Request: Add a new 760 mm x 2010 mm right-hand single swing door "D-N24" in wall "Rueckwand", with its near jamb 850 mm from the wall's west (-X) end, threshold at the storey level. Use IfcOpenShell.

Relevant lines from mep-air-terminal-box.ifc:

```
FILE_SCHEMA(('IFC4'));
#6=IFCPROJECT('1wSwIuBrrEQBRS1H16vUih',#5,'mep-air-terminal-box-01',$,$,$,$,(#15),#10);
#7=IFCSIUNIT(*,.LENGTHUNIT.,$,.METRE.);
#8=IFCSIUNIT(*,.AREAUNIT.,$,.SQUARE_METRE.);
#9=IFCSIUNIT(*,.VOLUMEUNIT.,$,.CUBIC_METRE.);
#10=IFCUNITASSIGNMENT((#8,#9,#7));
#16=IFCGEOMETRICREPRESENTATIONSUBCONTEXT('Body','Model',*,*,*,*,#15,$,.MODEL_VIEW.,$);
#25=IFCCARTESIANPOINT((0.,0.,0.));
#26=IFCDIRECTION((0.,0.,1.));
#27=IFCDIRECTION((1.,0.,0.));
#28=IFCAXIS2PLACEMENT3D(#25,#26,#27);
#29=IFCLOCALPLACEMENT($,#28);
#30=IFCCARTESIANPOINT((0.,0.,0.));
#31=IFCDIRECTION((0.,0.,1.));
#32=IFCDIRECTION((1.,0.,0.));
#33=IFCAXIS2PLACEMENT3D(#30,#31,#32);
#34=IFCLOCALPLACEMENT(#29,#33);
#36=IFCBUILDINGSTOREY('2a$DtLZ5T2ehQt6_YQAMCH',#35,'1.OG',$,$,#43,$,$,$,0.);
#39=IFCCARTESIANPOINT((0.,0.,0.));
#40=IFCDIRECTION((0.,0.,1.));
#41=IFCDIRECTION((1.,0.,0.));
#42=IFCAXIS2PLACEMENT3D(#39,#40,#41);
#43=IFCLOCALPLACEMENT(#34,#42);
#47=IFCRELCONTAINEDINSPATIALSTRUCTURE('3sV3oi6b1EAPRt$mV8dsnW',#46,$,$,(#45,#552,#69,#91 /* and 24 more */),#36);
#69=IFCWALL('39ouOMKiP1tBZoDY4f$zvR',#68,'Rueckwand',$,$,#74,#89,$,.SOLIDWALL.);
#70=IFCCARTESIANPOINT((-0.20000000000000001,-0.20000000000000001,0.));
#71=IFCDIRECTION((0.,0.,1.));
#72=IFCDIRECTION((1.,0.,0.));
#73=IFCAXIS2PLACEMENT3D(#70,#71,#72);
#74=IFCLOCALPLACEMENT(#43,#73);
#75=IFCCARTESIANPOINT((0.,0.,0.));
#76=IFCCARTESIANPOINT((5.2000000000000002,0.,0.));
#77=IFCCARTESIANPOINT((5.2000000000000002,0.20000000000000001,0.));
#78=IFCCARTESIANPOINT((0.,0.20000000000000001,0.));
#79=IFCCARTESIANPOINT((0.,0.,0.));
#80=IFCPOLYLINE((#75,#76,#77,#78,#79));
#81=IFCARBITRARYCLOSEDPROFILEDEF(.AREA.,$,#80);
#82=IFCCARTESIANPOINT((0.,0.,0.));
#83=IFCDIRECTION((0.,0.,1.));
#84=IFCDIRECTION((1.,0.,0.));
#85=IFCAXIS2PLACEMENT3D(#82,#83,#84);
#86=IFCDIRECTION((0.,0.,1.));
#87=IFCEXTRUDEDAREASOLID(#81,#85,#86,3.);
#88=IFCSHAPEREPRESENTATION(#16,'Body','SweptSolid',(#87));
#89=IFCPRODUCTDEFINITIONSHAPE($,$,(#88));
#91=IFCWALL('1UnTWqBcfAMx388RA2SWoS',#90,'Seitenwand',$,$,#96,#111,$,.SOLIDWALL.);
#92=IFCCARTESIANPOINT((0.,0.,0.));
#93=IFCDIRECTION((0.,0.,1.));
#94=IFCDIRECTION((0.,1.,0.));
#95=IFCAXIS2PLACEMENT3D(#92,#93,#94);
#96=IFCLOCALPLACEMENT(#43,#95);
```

```python
import numpy as np
import ifcopenshell
import ifcopenshell.api.feature
import ifcopenshell.api.geometry
import ifcopenshell.api.root
import ifcopenshell.api.spatial
import ifcopenshell.geom
import ifcopenshell.util.element
import ifcopenshell.util.placement
import ifcopenshell.util.representation
import ifcopenshell.util.shape
import ifcopenshell.util.unit

model = ifcopenshell.open("mep-air-terminal-box.ifc")
unit_scale = ifcopenshell.util.unit.calculate_unit_scale(model)
settings = ifcopenshell.geom.settings()


def volume(element):
    """Net volume in cubic metres, openings subtracted."""
    shape = ifcopenshell.geom.create_shape(settings, element)
    return ifcopenshell.util.shape.get_volume(shape.geometry)


wall = model.by_id(69)
storey = ifcopenshell.util.element.get_container(wall, ifc_class="IfcBuildingStorey")
context = ifcopenshell.util.representation.get_context(model, "Model", "Body", "MODEL_VIEW")
before = volume(wall)

width, height, from_end, sill = 0.76, 2.01, 0.85, 0.0  # metres

# The wall runs along its own X axis, and the end named is its -X end.
wall_shape = ifcopenshell.geom.create_shape(settings, wall)
x, y, z = ifcopenshell.util.shape.get_vertices(wall_shape.geometry).T
start = x.min() + from_end
face, thickness = float(y.min()), float(y.max() - y.min())
wall_matrix = ifcopenshell.util.placement.get_local_placement(wall.ObjectPlacement)
level = ifcopenshell.util.placement.get_local_placement(storey.ObjectPlacement)[2, 3]


def in_wall(x, y):
    """Placement at x, y metres in the wall's axes, at sill height."""
    matrix = wall_matrix.copy()
    matrix[:, 3] = wall_matrix @ np.array([x / unit_scale, y / unit_scale, 0.0, 1.0])
    matrix[2, 3] = level + sill / unit_scale
    return matrix


# Opening: a box that overshoots both wall faces by 50 mm.
opening = ifcopenshell.api.root.create_entity(model, ifc_class="IfcOpeningElement", predefined_type="OPENING")
box = ifcopenshell.api.geometry.add_wall_representation(
    model, context=context, length=width, height=height, thickness=thickness + 0.1
)
ifcopenshell.api.geometry.assign_representation(model, product=opening, representation=box)
ifcopenshell.api.geometry.edit_object_placement(model, product=opening, matrix=in_wall(start, face - 0.05), is_si=False)
ifcopenshell.api.feature.add_feature(model, feature=opening, element=wall)

door = ifcopenshell.api.root.create_entity(model, ifc_class="IfcDoor", name="D-N24", predefined_type="DOOR")
door.OverallWidth, door.OverallHeight = width / unit_scale, height / unit_scale
door.OperationType = "SINGLE_SWING_RIGHT"
body = ifcopenshell.api.geometry.add_door_representation(
    model,
    context=context,
    overall_width=door.OverallWidth,
    overall_height=door.OverallHeight,
    operation_type="SINGLE_SWING_RIGHT",
    lining_properties={"LiningDepth": thickness / unit_scale, "ThresholdDepth": thickness / unit_scale},
)
ifcopenshell.api.geometry.assign_representation(model, product=door, representation=body)
ifcopenshell.api.spatial.assign_container(model, products=[door], relating_structure=storey)
ifcopenshell.api.feature.add_filling(model, opening=opening, element=door)

# The lining spans the wall, so the door starts at the wall face.
ifcopenshell.api.geometry.edit_object_placement(model, product=door, matrix=in_wall(start, face), is_si=False)

after = volume(wall)

print(f"wall volume {before:.3f} -> {after:.3f} m3")

model.write("mep-air-terminal-box_rev.ifc")
```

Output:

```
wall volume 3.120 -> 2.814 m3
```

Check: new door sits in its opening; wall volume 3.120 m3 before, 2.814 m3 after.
